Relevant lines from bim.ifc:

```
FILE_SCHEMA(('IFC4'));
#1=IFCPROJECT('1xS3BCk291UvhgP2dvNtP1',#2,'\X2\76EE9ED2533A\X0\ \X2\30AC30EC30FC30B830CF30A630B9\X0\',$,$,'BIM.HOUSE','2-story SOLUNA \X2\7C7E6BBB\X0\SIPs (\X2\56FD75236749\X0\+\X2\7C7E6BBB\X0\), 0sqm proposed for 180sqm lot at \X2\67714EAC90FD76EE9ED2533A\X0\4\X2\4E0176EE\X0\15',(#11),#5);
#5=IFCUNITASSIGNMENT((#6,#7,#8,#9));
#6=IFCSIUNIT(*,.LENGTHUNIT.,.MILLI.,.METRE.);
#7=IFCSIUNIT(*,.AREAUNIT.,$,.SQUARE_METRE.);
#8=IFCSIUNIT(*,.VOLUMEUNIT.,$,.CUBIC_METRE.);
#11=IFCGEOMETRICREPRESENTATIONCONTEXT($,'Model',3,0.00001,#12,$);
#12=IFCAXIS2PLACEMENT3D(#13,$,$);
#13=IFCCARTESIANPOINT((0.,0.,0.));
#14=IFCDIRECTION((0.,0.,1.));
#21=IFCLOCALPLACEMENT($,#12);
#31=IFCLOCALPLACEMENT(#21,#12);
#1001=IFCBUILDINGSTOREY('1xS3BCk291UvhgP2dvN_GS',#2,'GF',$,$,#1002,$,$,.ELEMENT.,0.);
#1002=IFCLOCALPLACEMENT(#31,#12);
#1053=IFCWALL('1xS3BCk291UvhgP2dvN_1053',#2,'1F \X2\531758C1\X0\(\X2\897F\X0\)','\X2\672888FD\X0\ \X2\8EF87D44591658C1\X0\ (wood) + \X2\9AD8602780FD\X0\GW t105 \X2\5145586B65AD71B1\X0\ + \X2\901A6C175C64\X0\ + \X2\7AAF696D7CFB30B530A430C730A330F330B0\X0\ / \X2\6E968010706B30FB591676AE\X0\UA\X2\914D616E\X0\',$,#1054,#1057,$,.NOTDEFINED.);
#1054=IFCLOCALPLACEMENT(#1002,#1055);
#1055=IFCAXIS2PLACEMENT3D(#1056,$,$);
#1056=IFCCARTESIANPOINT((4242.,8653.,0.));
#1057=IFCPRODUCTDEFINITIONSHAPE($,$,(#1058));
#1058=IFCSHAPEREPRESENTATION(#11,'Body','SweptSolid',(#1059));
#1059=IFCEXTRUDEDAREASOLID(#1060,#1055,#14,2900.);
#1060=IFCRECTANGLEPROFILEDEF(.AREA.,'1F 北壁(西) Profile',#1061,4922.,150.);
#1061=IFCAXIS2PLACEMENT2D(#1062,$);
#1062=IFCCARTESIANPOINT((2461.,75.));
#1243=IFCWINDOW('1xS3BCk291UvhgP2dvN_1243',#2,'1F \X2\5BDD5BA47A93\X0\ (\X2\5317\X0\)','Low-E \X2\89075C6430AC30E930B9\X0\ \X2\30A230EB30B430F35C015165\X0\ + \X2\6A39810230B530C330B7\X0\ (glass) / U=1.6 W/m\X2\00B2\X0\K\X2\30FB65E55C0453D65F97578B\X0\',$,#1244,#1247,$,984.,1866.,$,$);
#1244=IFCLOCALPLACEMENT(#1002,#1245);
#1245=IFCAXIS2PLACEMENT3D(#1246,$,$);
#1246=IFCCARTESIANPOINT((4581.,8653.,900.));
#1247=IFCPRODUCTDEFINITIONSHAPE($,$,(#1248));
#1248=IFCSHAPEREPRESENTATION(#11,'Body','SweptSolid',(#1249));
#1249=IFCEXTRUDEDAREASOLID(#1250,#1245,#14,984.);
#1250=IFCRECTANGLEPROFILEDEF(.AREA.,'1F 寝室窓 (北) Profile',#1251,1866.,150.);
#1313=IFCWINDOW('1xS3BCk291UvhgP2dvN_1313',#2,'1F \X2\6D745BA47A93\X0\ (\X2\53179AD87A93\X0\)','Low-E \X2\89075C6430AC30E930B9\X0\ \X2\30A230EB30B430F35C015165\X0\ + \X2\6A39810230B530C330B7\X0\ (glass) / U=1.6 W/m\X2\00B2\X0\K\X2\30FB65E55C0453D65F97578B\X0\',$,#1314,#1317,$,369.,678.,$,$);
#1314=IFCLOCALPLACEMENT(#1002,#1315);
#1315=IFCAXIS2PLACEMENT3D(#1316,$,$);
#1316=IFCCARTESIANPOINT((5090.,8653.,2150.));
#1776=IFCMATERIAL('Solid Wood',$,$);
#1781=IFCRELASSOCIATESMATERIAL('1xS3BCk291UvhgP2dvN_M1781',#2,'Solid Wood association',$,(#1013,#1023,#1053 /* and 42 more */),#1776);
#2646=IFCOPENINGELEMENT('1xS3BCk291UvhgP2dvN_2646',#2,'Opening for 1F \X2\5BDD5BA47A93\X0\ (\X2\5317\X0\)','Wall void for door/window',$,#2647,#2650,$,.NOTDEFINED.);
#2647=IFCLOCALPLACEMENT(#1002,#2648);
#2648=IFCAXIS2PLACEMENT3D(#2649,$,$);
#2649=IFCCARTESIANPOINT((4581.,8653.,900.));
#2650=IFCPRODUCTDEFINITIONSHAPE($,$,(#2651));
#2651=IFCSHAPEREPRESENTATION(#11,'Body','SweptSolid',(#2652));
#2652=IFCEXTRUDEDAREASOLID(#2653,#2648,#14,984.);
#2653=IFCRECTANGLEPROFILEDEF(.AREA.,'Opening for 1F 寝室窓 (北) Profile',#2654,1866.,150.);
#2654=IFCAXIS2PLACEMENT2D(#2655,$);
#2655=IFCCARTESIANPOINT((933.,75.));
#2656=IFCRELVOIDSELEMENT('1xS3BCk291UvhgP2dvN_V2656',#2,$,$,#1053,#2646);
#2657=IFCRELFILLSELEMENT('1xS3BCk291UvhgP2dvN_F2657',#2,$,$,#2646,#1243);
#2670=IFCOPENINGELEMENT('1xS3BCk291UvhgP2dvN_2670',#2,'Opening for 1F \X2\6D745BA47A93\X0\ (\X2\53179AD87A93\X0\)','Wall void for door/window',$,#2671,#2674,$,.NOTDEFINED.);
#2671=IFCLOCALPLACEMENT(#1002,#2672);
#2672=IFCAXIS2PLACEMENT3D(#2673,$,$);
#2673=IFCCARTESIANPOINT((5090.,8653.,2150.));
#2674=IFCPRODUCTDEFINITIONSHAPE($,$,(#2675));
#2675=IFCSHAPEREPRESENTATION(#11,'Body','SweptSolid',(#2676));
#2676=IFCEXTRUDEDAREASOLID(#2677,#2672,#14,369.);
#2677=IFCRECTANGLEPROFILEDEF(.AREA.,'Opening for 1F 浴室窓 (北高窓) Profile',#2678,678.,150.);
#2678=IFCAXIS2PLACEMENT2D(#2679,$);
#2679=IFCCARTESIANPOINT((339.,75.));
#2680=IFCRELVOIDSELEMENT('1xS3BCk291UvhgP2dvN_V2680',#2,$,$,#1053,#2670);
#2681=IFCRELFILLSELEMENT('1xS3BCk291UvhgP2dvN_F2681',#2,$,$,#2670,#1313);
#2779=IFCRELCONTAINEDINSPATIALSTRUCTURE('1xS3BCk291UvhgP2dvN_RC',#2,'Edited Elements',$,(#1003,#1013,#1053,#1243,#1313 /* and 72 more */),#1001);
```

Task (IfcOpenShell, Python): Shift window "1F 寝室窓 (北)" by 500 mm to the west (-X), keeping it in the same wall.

```python
import ifcopenshell
import ifcopenshell.api.geometry
import ifcopenshell.util.placement
import ifcopenshell.util.unit

model = ifcopenshell.open("bim.ifc")
unit_scale = ifcopenshell.util.unit.calculate_unit_scale(model)

window = model.by_guid("1xS3BCk291UvhgP2dvN_1243")
opening = window.FillsVoids[0].RelatingOpeningElement
wall = opening.VoidsElements[0].RelatingBuildingElement

wall_matrix = ifcopenshell.util.placement.get_local_placement(wall.ObjectPlacement)
shift = wall_matrix[:3, 0] * -0.5 / unit_scale
before = ifcopenshell.util.placement.get_local_placement(window.ObjectPlacement)[:3, 3].copy()

# The window is not placed relative to its opening, so move both.
for product in (opening, window):
    matrix = ifcopenshell.util.placement.get_local_placement(product.ObjectPlacement)
    matrix[:3, 3] += shift
    ifcopenshell.api.geometry.edit_object_placement(model, product=product, matrix=matrix, is_si=False)

after = ifcopenshell.util.placement.get_local_placement(window.ObjectPlacement)[:3, 3]
print("window moved by", (after - before).round(3) + 0.0)

model.write("bim_updated.ifc")
```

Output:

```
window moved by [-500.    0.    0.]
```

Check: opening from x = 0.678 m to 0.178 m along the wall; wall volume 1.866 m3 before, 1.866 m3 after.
